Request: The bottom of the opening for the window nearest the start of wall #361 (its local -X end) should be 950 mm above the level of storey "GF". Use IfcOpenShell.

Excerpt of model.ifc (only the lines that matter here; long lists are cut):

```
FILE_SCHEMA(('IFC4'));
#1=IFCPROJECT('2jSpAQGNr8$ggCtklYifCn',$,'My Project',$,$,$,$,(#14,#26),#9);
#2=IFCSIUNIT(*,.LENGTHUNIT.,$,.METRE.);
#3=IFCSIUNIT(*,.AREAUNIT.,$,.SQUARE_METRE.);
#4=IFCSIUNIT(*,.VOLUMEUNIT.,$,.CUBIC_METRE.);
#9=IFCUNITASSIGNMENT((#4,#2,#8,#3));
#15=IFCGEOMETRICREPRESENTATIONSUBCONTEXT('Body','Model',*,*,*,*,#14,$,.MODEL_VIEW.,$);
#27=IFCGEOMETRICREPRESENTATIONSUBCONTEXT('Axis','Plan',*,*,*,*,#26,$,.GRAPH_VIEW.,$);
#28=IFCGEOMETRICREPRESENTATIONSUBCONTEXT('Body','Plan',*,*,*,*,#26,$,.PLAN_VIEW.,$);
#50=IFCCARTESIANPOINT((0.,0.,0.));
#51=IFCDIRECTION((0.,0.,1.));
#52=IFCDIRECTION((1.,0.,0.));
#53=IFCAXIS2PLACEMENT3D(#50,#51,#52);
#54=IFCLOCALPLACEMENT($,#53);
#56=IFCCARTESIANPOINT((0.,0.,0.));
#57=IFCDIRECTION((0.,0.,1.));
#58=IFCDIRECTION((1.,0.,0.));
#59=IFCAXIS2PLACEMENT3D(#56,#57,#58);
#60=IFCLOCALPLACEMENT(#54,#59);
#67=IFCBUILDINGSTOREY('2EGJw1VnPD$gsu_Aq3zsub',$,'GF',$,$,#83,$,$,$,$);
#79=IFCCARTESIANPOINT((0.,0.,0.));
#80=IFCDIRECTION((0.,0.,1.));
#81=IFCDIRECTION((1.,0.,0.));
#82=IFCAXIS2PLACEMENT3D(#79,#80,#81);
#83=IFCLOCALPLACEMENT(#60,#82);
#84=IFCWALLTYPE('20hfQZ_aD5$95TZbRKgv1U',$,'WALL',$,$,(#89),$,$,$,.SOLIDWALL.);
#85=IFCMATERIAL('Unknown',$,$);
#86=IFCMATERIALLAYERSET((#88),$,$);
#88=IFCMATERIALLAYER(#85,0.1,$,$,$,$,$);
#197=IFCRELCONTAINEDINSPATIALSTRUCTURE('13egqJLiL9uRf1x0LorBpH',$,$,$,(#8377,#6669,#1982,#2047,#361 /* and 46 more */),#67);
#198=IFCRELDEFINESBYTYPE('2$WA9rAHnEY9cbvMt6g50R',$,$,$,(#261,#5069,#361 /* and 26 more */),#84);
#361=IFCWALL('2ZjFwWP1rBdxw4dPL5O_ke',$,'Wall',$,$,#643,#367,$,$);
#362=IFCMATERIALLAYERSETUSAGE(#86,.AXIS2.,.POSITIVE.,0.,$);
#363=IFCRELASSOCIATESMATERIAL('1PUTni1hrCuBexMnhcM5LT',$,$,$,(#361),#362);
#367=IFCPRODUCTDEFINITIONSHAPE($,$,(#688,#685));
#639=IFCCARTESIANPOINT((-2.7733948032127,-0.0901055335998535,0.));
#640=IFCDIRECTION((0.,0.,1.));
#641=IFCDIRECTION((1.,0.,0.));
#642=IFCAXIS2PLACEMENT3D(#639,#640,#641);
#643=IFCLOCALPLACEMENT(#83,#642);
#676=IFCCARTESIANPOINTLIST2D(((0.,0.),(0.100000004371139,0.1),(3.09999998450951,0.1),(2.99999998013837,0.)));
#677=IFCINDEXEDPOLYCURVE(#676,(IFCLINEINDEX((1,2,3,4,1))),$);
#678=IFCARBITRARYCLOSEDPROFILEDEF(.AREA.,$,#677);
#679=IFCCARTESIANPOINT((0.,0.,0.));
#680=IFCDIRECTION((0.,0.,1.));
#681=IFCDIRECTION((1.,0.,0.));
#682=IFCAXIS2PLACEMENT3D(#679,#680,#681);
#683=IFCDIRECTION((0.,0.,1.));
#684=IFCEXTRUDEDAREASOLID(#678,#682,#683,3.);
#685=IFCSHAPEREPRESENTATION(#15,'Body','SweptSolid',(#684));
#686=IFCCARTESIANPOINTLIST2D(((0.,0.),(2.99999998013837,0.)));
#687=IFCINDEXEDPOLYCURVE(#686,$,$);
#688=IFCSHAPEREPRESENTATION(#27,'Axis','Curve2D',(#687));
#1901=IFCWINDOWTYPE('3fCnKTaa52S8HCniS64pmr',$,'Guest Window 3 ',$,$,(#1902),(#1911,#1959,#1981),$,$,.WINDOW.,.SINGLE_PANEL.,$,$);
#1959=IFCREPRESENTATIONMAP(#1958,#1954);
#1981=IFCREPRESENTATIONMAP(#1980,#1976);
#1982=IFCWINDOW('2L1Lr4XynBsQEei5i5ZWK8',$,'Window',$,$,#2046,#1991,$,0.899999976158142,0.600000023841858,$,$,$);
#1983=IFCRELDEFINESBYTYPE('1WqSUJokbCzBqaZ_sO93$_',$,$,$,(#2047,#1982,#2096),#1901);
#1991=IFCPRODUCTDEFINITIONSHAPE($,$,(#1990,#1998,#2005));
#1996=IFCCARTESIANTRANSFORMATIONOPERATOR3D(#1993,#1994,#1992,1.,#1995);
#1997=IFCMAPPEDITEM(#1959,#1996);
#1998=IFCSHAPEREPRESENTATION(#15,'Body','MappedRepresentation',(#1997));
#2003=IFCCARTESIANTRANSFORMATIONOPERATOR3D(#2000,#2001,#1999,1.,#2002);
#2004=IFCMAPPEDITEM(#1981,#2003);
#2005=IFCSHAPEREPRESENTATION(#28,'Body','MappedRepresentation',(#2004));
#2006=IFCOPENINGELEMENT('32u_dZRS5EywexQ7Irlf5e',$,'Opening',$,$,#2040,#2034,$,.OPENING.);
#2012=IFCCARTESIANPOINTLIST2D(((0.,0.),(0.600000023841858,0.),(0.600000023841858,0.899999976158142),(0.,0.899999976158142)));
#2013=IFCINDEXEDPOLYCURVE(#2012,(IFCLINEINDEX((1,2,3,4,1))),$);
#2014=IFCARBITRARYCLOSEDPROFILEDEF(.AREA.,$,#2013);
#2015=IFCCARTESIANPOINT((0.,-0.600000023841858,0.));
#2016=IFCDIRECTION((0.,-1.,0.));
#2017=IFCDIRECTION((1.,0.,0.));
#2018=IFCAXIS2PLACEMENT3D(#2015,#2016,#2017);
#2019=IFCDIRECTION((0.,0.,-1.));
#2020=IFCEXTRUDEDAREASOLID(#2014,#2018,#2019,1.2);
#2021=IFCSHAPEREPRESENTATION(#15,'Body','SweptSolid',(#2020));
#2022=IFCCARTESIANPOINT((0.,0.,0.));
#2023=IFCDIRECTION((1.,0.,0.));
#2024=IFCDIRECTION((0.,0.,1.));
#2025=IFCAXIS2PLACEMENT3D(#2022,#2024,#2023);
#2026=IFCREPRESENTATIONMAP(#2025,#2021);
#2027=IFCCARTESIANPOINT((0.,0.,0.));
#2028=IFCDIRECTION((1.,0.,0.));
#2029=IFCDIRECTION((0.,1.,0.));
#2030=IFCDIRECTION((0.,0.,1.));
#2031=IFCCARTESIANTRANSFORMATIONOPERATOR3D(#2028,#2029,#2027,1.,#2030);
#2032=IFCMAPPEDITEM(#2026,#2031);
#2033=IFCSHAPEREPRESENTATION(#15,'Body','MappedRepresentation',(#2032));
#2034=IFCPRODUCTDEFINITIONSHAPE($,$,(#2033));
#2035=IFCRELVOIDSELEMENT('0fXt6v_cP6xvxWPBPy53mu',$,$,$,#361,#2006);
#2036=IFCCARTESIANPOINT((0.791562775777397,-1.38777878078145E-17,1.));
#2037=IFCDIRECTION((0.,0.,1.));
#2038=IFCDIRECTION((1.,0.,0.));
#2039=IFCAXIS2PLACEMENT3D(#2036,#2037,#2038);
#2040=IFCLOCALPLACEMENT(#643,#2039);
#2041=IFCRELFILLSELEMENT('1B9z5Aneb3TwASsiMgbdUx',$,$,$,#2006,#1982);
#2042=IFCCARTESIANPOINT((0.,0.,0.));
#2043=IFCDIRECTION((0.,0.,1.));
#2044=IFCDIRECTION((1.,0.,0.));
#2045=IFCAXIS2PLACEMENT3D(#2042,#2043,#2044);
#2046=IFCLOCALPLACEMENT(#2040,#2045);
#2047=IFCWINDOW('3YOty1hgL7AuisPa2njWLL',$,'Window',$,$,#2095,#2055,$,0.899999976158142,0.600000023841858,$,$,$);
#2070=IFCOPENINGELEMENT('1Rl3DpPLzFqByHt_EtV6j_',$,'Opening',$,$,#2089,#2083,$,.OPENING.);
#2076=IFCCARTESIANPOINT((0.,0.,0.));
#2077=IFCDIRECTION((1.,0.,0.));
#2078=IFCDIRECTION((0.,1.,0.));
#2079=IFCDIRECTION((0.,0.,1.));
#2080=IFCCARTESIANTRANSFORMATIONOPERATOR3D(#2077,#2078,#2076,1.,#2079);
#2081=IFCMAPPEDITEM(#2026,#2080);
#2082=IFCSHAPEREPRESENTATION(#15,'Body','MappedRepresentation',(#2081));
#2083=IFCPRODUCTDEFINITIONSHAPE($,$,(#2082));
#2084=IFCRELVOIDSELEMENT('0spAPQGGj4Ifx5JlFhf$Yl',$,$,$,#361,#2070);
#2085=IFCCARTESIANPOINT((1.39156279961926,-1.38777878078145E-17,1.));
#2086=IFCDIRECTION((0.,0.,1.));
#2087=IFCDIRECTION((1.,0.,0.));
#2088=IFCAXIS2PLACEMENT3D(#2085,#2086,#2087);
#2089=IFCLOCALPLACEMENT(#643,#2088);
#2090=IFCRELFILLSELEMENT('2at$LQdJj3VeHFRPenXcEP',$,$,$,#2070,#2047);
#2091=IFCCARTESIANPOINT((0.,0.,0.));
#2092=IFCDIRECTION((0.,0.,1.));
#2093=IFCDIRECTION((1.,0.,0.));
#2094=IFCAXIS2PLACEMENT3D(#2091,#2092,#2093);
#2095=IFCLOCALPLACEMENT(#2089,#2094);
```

```python
import numpy as np
import ifcopenshell
import ifcopenshell.api.geometry
import ifcopenshell.geom
import ifcopenshell.util.element
import ifcopenshell.util.placement
import ifcopenshell.util.shape
import ifcopenshell.util.unit

model = ifcopenshell.open("model.ifc")
unit_scale = ifcopenshell.util.unit.calculate_unit_scale(model)

window = model.by_guid("2L1Lr4XynBsQEei5i5ZWK8")
opening = window.FillsVoids[0].RelatingOpeningElement
storey = ifcopenshell.util.element.get_container(window, ifc_class="IfcBuildingStorey")
level = ifcopenshell.util.placement.get_local_placement(storey.ObjectPlacement)[2, 3]

# The opening's origin need not be at the sill, so measure its lowest point.
shape = ifcopenshell.geom.create_shape(ifcopenshell.geom.settings(), opening)
bottom = ifcopenshell.util.shape.get_shape_bottom_elevation(shape, shape.geometry) / unit_scale
dz = level + 0.95 - bottom

shift = np.array([0.0, 0.0, dz])
# The window is placed relative to its opening, so it follows when the opening moves.
matrix = ifcopenshell.util.placement.get_local_placement(opening.ObjectPlacement)
matrix[:3, 3] += shift
ifcopenshell.api.geometry.edit_object_placement(
    model, product=opening, matrix=matrix, is_si=False, should_transform_children=True
)

print(f"moved by {dz * unit_scale:+.3f} m")

model.write("model_v2.ifc")
```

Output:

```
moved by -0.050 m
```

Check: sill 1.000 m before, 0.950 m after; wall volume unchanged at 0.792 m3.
